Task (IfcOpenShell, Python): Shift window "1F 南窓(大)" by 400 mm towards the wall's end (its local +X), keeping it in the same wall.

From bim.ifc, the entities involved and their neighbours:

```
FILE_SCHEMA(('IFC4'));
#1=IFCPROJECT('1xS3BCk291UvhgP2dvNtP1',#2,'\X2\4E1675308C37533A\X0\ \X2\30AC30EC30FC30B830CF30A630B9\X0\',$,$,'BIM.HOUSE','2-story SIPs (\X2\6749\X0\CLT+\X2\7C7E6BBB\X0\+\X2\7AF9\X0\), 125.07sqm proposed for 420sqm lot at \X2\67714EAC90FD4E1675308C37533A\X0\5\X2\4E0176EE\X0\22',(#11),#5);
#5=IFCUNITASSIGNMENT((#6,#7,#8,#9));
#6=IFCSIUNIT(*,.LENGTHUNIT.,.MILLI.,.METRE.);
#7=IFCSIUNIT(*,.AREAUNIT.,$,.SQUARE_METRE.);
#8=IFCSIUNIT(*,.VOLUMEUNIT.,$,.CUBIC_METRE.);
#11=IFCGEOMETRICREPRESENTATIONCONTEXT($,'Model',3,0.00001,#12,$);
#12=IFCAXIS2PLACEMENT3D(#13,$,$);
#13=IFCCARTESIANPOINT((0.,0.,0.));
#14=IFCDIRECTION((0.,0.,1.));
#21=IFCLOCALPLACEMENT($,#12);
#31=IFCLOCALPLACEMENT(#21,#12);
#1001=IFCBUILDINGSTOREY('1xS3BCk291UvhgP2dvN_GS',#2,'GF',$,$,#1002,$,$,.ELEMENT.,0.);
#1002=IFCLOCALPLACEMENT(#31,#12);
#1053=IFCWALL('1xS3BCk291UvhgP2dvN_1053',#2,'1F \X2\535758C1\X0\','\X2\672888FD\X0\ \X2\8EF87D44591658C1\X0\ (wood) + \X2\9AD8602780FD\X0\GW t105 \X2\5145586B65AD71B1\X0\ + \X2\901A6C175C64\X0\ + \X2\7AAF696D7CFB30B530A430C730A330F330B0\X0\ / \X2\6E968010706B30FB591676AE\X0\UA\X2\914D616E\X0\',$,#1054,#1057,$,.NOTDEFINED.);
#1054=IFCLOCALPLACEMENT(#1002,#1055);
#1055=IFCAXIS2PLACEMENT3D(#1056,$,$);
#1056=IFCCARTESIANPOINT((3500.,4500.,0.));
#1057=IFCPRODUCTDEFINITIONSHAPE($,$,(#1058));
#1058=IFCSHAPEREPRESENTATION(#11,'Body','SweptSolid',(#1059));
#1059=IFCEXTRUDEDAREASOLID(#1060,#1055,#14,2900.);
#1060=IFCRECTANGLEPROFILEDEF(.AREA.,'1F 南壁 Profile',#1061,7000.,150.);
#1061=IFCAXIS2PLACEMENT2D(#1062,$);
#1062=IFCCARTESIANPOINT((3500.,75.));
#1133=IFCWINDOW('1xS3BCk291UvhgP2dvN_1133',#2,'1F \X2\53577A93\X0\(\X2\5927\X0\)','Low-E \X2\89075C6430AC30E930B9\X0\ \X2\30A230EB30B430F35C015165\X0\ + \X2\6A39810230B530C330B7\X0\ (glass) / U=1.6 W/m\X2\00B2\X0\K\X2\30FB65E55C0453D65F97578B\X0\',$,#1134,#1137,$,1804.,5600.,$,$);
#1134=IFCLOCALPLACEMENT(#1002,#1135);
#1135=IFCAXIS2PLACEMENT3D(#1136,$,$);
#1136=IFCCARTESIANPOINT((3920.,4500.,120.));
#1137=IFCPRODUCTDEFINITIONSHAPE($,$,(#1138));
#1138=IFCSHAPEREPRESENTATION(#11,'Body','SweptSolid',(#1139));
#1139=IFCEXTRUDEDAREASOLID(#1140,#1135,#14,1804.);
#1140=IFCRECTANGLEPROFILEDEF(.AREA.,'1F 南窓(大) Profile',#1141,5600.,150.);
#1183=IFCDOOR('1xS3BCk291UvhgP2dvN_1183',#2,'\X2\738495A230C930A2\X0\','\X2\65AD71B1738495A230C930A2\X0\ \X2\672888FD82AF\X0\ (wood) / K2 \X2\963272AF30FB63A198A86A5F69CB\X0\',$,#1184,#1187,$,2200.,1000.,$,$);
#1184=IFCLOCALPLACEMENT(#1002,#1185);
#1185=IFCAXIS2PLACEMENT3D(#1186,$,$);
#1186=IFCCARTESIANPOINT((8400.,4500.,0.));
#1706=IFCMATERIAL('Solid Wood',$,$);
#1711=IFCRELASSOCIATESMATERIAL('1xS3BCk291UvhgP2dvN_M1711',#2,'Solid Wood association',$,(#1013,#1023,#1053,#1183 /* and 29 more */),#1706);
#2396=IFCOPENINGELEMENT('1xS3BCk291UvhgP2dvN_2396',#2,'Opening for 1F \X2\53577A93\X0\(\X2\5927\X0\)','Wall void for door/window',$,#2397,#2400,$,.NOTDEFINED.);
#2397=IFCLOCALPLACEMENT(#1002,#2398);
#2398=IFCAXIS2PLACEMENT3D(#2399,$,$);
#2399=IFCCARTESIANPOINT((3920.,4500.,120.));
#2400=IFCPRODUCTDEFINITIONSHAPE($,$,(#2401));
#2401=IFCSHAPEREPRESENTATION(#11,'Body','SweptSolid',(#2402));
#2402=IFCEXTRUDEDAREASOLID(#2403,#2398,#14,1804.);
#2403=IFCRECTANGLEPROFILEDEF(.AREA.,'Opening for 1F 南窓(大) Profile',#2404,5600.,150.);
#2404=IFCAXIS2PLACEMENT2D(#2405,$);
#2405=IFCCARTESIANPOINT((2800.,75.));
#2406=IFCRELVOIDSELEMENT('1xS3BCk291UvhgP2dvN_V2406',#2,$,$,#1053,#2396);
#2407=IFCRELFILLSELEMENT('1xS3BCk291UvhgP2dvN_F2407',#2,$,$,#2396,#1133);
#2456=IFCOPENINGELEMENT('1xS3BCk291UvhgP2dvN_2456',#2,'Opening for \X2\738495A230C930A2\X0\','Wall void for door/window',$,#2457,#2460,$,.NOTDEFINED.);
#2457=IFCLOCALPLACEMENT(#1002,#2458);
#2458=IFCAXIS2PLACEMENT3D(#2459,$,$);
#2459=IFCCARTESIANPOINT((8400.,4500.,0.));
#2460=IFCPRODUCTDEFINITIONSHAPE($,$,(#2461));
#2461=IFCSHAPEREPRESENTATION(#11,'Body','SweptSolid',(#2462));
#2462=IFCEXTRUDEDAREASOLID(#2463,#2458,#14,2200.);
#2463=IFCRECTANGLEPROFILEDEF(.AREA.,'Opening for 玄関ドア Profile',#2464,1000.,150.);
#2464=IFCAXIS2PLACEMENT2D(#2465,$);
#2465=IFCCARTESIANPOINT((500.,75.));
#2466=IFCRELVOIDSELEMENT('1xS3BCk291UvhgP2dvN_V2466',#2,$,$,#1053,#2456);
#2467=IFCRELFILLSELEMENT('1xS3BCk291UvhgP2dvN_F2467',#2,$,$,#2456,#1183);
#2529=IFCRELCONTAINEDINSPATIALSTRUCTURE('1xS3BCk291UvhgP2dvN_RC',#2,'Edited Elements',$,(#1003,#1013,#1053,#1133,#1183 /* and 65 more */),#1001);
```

```python
import ifcopenshell
import ifcopenshell.api.geometry
import ifcopenshell.util.placement
import ifcopenshell.util.unit

model = ifcopenshell.open("bim.ifc")
unit_scale = ifcopenshell.util.unit.calculate_unit_scale(model)

window = model.by_id(1133)
opening = window.FillsVoids[0].RelatingOpeningElement
wall = opening.VoidsElements[0].RelatingBuildingElement

wall_matrix = ifcopenshell.util.placement.get_local_placement(wall.ObjectPlacement)
shift = wall_matrix[:3, 0] * 0.4 / unit_scale
before = ifcopenshell.util.placement.get_local_placement(window.ObjectPlacement)[:3, 3].copy()

# The window is not placed relative to its opening, so move both.
for product in (opening, window):
    matrix = ifcopenshell.util.placement.get_local_placement(product.ObjectPlacement)
    matrix[:3, 3] += shift
    ifcopenshell.api.geometry.edit_object_placement(model, product=product, matrix=matrix, is_si=False)

after = ifcopenshell.util.placement.get_local_placement(window.ObjectPlacement)[:3, 3]
print("window moved by", (after - before).round(3) + 0.0)

model.write("bim_rev.ifc")
```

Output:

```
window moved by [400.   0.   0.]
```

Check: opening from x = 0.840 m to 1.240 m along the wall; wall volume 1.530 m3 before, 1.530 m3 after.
